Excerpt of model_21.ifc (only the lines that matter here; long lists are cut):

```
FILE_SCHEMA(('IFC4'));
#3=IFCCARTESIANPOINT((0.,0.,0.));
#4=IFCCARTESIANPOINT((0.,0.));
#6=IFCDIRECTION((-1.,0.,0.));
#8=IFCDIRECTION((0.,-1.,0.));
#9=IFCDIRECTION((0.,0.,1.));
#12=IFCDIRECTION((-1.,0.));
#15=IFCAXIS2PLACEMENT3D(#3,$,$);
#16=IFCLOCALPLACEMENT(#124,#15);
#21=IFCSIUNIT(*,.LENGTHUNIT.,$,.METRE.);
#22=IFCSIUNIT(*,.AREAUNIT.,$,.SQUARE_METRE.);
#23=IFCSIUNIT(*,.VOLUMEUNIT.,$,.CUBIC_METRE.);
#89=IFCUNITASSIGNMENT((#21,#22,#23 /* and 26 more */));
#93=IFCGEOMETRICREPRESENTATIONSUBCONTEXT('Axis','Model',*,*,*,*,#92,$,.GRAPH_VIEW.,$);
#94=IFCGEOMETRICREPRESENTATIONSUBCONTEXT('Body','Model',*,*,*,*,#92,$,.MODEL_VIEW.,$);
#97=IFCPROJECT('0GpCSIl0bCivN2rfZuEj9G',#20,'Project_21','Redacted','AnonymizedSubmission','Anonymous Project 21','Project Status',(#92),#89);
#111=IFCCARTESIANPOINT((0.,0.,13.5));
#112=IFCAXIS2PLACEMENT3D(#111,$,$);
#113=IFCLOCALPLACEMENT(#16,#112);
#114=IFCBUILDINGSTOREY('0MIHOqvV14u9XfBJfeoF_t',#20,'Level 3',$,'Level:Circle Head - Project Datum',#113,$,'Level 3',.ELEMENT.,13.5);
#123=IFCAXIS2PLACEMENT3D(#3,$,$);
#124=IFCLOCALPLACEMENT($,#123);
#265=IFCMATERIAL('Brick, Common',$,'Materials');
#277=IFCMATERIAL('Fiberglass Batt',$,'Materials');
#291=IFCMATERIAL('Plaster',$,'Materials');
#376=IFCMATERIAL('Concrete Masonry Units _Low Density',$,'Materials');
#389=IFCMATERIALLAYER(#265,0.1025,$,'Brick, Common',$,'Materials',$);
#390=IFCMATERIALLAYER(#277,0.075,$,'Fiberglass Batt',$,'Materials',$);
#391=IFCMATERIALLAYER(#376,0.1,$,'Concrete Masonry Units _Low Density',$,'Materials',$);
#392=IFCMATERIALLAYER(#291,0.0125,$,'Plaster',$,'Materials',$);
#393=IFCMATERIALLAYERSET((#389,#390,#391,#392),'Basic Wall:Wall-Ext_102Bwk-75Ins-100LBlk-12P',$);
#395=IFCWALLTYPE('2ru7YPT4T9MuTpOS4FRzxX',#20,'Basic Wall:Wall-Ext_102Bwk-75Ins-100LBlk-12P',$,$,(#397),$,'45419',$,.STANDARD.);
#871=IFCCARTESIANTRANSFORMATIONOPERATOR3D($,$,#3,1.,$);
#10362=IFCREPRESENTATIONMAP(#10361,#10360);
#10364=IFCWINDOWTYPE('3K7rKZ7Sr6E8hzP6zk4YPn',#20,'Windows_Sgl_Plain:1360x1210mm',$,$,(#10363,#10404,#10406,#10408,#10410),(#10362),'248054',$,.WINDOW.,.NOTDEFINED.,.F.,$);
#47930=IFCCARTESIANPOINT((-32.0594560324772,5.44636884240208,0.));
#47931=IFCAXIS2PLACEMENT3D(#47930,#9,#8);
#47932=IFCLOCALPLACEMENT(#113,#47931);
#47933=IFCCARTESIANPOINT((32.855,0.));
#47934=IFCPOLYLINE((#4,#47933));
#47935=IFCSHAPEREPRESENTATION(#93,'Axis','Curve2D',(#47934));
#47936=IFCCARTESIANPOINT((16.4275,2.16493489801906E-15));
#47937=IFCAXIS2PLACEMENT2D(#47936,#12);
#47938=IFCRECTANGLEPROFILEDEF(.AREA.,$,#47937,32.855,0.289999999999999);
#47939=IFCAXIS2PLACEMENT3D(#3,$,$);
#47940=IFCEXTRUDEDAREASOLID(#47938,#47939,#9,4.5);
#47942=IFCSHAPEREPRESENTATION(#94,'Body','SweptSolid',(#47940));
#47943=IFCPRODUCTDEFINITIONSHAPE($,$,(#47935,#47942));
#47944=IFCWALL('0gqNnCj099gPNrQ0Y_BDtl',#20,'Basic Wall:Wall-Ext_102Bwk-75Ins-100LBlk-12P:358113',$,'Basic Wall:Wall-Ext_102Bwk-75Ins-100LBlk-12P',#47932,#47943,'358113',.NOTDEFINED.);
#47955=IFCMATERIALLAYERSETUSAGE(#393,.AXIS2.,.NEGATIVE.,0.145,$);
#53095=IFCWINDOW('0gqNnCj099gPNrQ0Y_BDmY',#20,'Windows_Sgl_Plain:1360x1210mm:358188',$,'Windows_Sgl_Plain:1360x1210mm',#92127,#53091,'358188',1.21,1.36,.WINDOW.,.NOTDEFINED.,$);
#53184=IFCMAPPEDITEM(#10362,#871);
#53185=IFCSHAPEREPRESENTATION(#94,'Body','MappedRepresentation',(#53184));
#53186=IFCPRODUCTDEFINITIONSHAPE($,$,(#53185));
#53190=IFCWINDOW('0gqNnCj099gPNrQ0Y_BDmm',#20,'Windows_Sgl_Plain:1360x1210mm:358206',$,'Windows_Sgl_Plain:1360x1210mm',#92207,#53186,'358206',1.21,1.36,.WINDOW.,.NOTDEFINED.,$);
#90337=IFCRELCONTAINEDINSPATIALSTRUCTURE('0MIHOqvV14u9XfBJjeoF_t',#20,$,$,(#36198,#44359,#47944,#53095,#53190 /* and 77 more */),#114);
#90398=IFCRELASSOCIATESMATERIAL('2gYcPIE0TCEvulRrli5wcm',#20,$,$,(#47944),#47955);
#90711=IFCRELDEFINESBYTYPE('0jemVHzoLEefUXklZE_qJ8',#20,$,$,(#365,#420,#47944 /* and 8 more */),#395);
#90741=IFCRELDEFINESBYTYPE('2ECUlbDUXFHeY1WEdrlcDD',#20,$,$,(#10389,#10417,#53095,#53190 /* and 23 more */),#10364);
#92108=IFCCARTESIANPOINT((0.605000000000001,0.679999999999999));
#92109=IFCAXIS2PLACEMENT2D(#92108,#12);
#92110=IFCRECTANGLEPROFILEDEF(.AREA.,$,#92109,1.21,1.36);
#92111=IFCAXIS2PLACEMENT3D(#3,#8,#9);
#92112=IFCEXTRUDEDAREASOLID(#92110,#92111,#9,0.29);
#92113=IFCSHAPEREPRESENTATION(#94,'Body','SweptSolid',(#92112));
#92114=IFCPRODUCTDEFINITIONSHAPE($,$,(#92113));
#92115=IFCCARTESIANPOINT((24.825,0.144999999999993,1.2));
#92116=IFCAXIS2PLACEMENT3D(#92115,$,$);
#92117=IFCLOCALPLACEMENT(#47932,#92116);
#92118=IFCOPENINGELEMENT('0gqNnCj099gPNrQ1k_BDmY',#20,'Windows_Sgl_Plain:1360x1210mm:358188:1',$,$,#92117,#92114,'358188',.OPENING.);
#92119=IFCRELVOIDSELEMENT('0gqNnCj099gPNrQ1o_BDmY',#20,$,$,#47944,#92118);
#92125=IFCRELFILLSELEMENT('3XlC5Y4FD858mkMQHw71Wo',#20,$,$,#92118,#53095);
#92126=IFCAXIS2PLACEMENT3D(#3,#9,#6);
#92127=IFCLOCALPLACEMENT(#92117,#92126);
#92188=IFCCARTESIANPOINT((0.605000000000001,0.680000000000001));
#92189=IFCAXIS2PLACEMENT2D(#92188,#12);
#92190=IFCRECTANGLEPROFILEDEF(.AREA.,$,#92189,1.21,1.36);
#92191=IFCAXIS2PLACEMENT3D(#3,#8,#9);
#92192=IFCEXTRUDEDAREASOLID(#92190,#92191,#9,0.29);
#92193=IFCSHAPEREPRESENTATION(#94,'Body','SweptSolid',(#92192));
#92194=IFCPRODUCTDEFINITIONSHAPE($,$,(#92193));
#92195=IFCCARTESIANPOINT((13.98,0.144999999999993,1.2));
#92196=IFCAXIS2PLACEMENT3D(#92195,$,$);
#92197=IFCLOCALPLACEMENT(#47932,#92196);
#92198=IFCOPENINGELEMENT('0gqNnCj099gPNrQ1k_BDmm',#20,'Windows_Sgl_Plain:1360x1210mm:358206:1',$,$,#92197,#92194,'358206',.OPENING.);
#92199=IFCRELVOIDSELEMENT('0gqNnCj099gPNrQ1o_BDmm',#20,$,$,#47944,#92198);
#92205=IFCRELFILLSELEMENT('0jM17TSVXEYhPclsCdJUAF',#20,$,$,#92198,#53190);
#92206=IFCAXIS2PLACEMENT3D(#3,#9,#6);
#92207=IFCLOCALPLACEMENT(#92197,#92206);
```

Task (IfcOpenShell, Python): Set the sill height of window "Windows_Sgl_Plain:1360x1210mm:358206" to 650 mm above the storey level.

```python
import numpy as np
import ifcopenshell
import ifcopenshell.api.geometry
import ifcopenshell.geom
import ifcopenshell.util.element
import ifcopenshell.util.placement
import ifcopenshell.util.shape
import ifcopenshell.util.unit

model = ifcopenshell.open("model_21.ifc")
unit_scale = ifcopenshell.util.unit.calculate_unit_scale(model)

window = model.by_guid("0gqNnCj099gPNrQ0Y_BDmm")
opening = window.FillsVoids[0].RelatingOpeningElement
storey = ifcopenshell.util.element.get_container(window, ifc_class="IfcBuildingStorey")
level = ifcopenshell.util.placement.get_local_placement(storey.ObjectPlacement)[2, 3]

# The opening's origin need not be at the sill, so measure its lowest point.
shape = ifcopenshell.geom.create_shape(ifcopenshell.geom.settings(), opening)
bottom = ifcopenshell.util.shape.get_shape_bottom_elevation(shape, shape.geometry) / unit_scale
dz = level + 0.65 / unit_scale - bottom

shift = np.array([0.0, 0.0, dz])
# The window is placed relative to its opening, so it follows when the opening moves.
matrix = ifcopenshell.util.placement.get_local_placement(opening.ObjectPlacement)
matrix[:3, 3] += shift
ifcopenshell.api.geometry.edit_object_placement(
    model, product=opening, matrix=matrix, is_si=False, should_transform_children=True
)

print(f"moved by {dz * unit_scale:+.3f} m")

model.write("model_21_rev.ifc")
```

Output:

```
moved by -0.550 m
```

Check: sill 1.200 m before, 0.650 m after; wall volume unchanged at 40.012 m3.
